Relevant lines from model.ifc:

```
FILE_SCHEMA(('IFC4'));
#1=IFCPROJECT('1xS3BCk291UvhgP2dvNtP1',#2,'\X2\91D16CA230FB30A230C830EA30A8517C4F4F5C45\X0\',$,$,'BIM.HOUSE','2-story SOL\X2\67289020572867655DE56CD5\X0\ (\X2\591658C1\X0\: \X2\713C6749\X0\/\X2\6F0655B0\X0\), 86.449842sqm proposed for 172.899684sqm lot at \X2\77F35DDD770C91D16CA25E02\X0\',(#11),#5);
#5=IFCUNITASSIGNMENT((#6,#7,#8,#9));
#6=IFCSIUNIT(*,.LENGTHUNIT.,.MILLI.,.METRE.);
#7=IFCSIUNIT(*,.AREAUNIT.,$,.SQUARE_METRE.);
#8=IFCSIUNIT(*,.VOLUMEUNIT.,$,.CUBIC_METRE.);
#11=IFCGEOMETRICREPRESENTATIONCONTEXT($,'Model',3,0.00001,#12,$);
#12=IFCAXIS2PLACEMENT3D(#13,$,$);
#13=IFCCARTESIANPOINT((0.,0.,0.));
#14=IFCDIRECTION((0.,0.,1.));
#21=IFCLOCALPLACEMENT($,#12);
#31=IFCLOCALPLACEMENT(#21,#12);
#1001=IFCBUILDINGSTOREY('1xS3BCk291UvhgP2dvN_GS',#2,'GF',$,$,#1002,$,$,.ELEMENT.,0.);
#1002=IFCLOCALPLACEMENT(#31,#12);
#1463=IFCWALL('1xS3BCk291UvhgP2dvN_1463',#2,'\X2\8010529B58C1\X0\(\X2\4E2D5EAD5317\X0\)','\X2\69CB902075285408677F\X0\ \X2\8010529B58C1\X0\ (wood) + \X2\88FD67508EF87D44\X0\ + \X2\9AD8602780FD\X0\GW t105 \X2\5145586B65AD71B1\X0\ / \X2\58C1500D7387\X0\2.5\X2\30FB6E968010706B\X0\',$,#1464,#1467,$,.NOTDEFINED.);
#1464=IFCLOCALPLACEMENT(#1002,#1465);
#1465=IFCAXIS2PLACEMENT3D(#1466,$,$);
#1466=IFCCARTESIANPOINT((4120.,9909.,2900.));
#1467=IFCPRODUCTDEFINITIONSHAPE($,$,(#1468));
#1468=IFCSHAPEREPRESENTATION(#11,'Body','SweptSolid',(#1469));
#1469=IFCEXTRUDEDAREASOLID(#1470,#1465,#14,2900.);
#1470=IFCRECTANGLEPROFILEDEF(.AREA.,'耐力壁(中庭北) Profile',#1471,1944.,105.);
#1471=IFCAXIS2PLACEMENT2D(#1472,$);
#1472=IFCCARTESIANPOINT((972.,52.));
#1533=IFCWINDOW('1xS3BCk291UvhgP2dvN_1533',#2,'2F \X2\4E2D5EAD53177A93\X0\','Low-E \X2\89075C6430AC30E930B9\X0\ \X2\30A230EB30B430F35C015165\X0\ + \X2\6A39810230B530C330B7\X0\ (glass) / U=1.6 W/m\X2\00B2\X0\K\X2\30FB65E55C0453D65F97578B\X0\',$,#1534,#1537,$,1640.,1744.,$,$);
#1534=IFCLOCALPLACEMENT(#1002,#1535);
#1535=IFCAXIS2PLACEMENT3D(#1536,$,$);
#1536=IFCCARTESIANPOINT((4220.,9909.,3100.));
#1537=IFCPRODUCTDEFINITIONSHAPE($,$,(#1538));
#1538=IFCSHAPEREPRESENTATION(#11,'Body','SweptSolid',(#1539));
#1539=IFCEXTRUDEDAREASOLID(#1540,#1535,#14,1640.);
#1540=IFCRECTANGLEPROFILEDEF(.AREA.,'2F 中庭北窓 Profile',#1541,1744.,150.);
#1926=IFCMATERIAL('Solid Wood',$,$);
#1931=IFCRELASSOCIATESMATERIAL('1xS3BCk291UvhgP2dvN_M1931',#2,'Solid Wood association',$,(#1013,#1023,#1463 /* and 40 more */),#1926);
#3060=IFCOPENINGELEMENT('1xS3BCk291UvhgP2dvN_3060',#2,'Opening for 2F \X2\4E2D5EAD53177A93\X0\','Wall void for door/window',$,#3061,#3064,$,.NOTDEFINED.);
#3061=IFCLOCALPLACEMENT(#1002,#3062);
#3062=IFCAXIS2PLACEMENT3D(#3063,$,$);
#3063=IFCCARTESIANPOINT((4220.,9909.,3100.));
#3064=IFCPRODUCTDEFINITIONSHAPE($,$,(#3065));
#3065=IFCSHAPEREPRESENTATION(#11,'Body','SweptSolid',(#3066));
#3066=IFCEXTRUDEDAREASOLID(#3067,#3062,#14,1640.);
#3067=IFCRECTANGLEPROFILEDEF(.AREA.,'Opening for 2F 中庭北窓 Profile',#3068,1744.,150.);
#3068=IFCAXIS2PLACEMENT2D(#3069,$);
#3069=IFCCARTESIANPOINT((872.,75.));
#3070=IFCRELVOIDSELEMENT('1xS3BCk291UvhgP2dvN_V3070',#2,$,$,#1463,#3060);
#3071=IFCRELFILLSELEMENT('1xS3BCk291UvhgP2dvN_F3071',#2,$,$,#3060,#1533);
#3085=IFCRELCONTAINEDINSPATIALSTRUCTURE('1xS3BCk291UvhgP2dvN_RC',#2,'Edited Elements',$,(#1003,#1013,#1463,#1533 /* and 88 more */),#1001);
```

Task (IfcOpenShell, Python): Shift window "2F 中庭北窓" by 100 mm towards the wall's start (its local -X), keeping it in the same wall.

```python
import ifcopenshell
import ifcopenshell.api.geometry
import ifcopenshell.util.placement
import ifcopenshell.util.unit

model = ifcopenshell.open("model.ifc")
unit_scale = ifcopenshell.util.unit.calculate_unit_scale(model)

window = model.by_id(1533)
opening = window.FillsVoids[0].RelatingOpeningElement
wall = opening.VoidsElements[0].RelatingBuildingElement

wall_matrix = ifcopenshell.util.placement.get_local_placement(wall.ObjectPlacement)
shift = wall_matrix[:3, 0] * -0.1 / unit_scale
before = ifcopenshell.util.placement.get_local_placement(window.ObjectPlacement)[:3, 3].copy()

# The window is not placed relative to its opening, so move both.
for product in (opening, window):
    matrix = ifcopenshell.util.placement.get_local_placement(product.ObjectPlacement)
    matrix[:3, 3] += shift
    ifcopenshell.api.geometry.edit_object_placement(model, product=product, matrix=matrix, is_si=False)

after = ifcopenshell.util.placement.get_local_placement(window.ObjectPlacement)[:3, 3]
print("window moved by", (after - before).round(3) + 0.0)

model.write("model_updated.ifc")
```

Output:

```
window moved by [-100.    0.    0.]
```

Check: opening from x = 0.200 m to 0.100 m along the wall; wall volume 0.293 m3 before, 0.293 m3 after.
